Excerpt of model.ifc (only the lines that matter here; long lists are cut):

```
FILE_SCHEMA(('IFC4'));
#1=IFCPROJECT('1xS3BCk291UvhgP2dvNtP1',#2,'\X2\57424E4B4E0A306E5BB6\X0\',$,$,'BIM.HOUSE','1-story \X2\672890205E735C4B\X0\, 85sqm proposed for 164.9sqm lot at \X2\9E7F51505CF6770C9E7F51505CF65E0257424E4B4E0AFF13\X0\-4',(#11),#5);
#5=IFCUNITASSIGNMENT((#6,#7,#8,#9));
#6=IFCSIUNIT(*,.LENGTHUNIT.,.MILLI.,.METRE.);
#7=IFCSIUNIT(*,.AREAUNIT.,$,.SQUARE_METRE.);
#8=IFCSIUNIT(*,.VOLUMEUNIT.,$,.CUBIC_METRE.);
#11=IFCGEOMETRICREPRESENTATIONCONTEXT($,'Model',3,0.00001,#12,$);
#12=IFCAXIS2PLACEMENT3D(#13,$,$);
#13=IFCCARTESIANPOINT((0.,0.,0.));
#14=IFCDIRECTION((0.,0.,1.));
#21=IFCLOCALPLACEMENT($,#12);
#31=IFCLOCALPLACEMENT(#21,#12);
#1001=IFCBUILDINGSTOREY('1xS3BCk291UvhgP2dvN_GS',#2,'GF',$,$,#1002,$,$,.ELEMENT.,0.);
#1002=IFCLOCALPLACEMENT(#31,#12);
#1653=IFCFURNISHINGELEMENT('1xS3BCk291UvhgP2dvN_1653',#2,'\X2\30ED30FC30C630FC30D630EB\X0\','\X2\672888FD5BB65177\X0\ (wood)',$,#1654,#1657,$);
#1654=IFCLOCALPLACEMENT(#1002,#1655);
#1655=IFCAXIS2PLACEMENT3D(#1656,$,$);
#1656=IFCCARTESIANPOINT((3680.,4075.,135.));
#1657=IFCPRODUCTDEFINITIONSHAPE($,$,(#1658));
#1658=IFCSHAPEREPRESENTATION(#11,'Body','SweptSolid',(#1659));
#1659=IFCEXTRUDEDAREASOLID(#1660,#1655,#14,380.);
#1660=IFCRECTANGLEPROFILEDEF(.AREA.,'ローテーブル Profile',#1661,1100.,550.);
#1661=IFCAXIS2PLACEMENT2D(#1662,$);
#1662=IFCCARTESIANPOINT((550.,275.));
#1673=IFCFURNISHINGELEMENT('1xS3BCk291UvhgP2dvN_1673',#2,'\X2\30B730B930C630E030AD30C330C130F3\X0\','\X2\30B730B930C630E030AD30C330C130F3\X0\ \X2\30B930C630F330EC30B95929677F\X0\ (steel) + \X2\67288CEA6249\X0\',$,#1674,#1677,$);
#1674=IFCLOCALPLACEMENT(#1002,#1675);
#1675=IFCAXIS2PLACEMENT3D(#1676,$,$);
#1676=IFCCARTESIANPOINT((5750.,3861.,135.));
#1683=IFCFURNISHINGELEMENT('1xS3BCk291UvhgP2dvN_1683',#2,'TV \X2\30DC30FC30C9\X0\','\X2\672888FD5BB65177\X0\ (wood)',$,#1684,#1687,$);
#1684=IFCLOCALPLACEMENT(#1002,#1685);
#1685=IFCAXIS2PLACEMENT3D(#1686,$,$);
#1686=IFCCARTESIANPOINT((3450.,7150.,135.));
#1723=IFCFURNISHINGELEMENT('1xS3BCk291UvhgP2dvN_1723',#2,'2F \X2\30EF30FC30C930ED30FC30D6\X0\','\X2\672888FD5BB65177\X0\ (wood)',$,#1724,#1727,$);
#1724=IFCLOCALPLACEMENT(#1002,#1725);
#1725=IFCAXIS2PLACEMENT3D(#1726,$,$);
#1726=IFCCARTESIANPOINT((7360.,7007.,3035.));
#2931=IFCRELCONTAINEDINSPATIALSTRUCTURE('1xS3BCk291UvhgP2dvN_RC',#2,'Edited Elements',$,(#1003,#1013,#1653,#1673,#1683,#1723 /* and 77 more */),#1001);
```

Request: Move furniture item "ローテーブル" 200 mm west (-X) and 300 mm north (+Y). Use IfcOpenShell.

```python
import ifcopenshell
import ifcopenshell.api.geometry
import ifcopenshell.util.placement
import ifcopenshell.util.unit

model = ifcopenshell.open("model.ifc")
unit_scale = ifcopenshell.util.unit.calculate_unit_scale(model)

item = model.by_id(1653)
matrix = ifcopenshell.util.placement.get_local_placement(item.ObjectPlacement)
matrix[0, 3] -= 0.2 / unit_scale
matrix[1, 3] += 0.3 / unit_scale
ifcopenshell.api.geometry.edit_object_placement(model, product=item, matrix=matrix, is_si=False)

print(ifcopenshell.util.placement.get_local_placement(item.ObjectPlacement).round(3) + 0.0)

model.write("model-out.ifc")
```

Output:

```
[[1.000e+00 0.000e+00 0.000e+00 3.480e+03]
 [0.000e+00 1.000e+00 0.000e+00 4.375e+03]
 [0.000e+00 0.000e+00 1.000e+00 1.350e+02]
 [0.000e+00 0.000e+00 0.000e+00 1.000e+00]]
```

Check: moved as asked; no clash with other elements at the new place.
